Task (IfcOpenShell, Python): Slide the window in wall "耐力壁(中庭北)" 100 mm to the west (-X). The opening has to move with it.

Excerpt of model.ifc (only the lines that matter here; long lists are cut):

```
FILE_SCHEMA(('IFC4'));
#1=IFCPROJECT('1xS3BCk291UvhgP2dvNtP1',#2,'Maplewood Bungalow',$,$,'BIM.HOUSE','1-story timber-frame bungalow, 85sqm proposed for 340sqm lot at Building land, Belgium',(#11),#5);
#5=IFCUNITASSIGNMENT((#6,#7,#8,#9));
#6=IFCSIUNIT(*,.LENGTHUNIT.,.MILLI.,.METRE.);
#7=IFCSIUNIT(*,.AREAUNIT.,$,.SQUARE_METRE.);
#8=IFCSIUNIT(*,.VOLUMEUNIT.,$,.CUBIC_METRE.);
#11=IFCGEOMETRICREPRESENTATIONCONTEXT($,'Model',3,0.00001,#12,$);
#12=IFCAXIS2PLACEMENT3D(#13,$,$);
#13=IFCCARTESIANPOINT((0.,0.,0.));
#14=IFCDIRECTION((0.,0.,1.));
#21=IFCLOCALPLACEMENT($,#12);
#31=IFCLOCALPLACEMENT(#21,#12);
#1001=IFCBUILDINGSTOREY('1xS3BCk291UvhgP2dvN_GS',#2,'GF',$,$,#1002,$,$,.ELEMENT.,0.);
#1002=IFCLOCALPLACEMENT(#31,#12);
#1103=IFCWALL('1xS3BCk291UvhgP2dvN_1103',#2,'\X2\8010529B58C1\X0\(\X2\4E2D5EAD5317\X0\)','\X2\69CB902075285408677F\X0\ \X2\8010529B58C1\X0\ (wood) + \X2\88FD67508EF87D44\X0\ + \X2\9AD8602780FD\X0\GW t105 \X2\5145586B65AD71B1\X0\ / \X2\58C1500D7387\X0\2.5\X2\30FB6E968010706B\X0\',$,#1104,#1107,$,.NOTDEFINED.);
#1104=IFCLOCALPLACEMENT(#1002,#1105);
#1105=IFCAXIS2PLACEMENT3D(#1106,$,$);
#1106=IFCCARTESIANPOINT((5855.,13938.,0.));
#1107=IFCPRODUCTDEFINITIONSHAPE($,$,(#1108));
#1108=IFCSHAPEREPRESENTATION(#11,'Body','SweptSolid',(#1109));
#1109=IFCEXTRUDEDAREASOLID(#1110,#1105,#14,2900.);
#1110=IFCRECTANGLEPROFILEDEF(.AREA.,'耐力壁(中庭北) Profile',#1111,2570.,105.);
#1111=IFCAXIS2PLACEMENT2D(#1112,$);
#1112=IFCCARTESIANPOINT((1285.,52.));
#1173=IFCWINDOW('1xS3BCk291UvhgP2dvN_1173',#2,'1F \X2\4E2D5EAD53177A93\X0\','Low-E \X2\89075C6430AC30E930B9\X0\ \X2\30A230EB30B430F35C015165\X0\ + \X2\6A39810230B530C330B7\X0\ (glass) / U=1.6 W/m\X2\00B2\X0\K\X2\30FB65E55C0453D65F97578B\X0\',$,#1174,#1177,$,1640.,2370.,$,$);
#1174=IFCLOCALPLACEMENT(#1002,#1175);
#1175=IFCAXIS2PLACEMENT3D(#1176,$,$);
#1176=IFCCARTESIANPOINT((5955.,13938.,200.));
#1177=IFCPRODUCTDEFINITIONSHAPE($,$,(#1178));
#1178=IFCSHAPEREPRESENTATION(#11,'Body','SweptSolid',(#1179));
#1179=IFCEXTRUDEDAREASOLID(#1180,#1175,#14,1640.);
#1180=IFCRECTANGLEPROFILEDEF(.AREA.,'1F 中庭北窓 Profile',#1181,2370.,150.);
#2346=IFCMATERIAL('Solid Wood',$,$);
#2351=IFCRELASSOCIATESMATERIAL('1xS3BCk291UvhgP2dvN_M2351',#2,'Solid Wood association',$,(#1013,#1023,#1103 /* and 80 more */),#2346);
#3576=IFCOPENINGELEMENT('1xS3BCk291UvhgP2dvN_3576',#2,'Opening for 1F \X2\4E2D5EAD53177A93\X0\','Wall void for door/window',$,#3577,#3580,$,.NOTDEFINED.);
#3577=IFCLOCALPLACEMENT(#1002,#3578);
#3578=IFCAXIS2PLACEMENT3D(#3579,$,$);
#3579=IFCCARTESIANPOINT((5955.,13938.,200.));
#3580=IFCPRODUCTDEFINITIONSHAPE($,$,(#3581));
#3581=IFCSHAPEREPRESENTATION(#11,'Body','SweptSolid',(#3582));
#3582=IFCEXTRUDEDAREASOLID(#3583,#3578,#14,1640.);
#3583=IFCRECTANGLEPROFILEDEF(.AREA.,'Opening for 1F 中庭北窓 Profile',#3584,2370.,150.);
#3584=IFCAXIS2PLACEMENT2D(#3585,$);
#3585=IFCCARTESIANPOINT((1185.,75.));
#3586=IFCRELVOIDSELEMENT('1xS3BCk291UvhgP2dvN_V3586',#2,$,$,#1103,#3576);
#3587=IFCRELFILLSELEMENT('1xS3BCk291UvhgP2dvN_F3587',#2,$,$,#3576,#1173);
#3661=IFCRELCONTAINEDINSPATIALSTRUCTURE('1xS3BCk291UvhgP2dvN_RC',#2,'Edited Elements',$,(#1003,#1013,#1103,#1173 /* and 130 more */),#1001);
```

```python
import ifcopenshell
import ifcopenshell.api.geometry
import ifcopenshell.util.placement
import ifcopenshell.util.unit

model = ifcopenshell.open("model.ifc")
unit_scale = ifcopenshell.util.unit.calculate_unit_scale(model)

window = model.by_guid("1xS3BCk291UvhgP2dvN_1173")
opening = window.FillsVoids[0].RelatingOpeningElement
wall = opening.VoidsElements[0].RelatingBuildingElement

wall_matrix = ifcopenshell.util.placement.get_local_placement(wall.ObjectPlacement)
shift = wall_matrix[:3, 0] * -0.1 / unit_scale
before = ifcopenshell.util.placement.get_local_placement(window.ObjectPlacement)[:3, 3].copy()

# The window is not placed relative to its opening, so move both.
for product in (opening, window):
    matrix = ifcopenshell.util.placement.get_local_placement(product.ObjectPlacement)
    matrix[:3, 3] += shift
    ifcopenshell.api.geometry.edit_object_placement(model, product=product, matrix=matrix, is_si=False)

after = ifcopenshell.util.placement.get_local_placement(window.ObjectPlacement)[:3, 3]
print("window moved by", (after - before).round(3) + 0.0)

model.write("model-out.ifc")
```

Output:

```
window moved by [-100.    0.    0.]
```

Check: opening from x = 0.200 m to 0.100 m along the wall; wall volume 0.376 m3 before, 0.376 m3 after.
